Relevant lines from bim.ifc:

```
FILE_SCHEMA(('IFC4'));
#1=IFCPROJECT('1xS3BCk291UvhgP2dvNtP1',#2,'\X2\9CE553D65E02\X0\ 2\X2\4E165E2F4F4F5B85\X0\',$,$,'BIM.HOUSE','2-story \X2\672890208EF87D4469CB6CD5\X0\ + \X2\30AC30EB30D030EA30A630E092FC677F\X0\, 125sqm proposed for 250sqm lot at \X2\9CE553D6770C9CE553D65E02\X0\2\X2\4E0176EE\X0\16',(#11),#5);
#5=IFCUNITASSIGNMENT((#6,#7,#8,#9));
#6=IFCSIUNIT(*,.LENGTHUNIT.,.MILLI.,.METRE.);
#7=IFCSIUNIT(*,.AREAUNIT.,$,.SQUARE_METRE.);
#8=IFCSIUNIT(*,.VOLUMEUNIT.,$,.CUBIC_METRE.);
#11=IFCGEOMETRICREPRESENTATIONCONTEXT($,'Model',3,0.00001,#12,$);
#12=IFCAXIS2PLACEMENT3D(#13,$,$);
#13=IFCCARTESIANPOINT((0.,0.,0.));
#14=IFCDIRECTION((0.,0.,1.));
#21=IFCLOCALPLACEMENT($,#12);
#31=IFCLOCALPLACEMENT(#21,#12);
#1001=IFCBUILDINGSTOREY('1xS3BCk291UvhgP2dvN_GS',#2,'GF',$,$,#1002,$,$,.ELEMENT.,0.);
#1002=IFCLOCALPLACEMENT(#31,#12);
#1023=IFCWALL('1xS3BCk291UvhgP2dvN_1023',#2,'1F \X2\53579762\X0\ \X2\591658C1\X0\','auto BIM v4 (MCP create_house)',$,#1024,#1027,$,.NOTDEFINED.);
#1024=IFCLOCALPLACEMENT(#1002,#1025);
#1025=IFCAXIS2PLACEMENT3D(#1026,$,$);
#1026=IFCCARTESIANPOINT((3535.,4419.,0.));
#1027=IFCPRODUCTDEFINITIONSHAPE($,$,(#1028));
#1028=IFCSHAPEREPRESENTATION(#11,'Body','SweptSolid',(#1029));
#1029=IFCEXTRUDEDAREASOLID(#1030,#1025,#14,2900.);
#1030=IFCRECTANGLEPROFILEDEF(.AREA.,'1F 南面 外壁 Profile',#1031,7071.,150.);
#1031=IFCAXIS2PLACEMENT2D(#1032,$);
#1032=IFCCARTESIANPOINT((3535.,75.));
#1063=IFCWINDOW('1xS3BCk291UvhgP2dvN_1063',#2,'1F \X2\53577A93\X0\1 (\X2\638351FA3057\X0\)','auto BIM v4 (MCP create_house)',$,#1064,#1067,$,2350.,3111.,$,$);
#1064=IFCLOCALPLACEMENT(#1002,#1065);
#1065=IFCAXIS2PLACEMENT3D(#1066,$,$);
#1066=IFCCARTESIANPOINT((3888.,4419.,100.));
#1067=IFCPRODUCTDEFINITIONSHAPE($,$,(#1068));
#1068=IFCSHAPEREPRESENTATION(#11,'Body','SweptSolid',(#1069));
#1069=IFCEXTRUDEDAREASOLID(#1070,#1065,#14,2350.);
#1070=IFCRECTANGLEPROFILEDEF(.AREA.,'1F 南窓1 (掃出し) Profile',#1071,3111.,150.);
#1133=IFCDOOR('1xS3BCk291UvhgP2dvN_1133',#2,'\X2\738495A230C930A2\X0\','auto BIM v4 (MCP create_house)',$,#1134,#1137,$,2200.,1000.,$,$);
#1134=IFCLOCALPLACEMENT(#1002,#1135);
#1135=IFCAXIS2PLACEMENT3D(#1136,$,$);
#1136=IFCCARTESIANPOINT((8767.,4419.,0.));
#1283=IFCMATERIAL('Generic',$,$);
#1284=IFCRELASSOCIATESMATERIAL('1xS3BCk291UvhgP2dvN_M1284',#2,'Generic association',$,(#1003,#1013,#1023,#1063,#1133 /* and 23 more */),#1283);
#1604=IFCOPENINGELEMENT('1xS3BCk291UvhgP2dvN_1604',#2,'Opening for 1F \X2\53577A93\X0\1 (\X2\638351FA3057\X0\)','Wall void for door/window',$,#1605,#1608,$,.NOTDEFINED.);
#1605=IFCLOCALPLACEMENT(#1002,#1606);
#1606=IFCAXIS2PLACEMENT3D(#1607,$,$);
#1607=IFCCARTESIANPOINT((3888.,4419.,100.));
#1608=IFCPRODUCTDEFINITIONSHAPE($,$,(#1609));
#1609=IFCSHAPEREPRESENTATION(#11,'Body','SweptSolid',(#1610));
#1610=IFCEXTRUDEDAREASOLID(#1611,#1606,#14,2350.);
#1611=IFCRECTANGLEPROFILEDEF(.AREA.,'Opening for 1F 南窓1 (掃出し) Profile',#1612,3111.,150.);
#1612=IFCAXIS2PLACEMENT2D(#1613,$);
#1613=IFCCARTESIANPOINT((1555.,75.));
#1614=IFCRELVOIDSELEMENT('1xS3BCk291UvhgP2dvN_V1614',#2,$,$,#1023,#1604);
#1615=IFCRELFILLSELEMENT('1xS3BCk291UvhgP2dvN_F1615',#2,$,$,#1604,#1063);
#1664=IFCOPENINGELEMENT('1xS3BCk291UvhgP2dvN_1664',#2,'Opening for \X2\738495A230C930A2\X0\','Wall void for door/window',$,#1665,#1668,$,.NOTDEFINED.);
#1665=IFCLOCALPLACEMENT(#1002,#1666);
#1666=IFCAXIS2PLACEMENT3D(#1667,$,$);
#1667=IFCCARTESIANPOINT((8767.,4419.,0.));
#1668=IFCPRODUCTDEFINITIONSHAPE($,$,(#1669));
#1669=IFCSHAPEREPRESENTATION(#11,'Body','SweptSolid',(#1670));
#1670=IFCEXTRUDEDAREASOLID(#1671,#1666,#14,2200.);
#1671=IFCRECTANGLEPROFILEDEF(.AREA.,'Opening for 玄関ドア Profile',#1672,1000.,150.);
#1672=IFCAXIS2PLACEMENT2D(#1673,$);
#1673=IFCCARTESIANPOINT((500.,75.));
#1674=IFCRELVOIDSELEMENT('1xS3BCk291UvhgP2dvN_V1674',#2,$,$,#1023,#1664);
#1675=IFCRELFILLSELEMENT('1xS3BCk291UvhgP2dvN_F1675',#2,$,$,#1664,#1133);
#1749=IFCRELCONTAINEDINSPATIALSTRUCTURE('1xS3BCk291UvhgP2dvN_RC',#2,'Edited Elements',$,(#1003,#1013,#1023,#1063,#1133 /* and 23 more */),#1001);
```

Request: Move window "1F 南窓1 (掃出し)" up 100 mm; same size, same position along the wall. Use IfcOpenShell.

```python
import numpy as np
import ifcopenshell
import ifcopenshell.api.geometry
import ifcopenshell.util.placement
import ifcopenshell.util.unit

model = ifcopenshell.open("bim.ifc")
unit_scale = ifcopenshell.util.unit.calculate_unit_scale(model)

window = model.by_guid("1xS3BCk291UvhgP2dvN_1063")
opening = window.FillsVoids[0].RelatingOpeningElement
dz = 0.1 / unit_scale

shift = np.array([0.0, 0.0, dz])
# The window is not placed relative to its opening, so move both.
for product in (opening, window):
    matrix = ifcopenshell.util.placement.get_local_placement(product.ObjectPlacement)
    matrix[:3, 3] += shift
    ifcopenshell.api.geometry.edit_object_placement(model, product=product, matrix=matrix, is_si=False)

print(f"moved by {dz * unit_scale:+.3f} m")

model.write("bim_v2.ifc")
```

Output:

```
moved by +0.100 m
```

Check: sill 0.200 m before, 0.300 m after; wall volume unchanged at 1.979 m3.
